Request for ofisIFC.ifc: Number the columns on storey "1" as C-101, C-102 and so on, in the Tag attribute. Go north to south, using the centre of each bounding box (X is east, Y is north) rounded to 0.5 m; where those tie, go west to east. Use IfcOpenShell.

First a look at what the model holds.

```python
import ifcopenshell
import ifcopenshell.util.element
import ifcopenshell.util.placement

model = ifcopenshell.open("ofisIFC.ifc")
print(model.schema)
storey = next(s for s in model.by_type("IfcBuildingStorey") if s.Name == "1")
columns = [e for e in ifcopenshell.util.element.get_decomposition(storey) if e.is_a("IfcColumn")]
for e in sorted(columns, key=lambda e: e.id()):
    origin = ifcopenshell.util.placement.get_local_placement(e.ObjectPlacement)[:3, 3]
    print(e.id(), e.Tag, e.Name, origin.round(2) + 0.0, sep=" | ")
```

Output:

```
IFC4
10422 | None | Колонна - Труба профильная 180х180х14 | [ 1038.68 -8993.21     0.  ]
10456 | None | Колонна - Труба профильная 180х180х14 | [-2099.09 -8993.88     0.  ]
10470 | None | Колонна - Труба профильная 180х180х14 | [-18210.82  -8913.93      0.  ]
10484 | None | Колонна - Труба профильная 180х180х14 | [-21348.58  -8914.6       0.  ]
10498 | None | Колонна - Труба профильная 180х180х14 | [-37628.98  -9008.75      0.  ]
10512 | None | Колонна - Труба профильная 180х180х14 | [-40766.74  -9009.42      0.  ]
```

```python
import ifcopenshell
import ifcopenshell.geom
import ifcopenshell.util.element
import ifcopenshell.util.shape

model = ifcopenshell.open("ofisIFC.ifc")
settings = ifcopenshell.geom.settings()
settings.set("use-world-coords", True)


def centre(element):
    shape = ifcopenshell.geom.create_shape(settings, element)
    return ifcopenshell.util.shape.get_bbox_centroid(shape.geometry)


storey = next(s for s in model.by_type("IfcBuildingStorey") if s.Name == "1")
columns = [e for e in ifcopenshell.util.element.get_decomposition(storey) if e.is_a("IfcColumn")]

# Insertion points can sit at a corner or the storey origin, so sort by the geometry (in metres).
centres = {e: centre(e) for e in columns}
columns.sort(key=lambda e: (-round(centres[e][1] / 0.5), centres[e][0]))

for i, e in enumerate(columns, start=1):
    number = f"C-1{i:02d}"
    e.Tag = number
    print(e.id(), number)

model.write("ofisIFC_updated.ifc")
```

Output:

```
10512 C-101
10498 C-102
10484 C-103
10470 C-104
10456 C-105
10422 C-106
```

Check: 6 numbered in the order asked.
